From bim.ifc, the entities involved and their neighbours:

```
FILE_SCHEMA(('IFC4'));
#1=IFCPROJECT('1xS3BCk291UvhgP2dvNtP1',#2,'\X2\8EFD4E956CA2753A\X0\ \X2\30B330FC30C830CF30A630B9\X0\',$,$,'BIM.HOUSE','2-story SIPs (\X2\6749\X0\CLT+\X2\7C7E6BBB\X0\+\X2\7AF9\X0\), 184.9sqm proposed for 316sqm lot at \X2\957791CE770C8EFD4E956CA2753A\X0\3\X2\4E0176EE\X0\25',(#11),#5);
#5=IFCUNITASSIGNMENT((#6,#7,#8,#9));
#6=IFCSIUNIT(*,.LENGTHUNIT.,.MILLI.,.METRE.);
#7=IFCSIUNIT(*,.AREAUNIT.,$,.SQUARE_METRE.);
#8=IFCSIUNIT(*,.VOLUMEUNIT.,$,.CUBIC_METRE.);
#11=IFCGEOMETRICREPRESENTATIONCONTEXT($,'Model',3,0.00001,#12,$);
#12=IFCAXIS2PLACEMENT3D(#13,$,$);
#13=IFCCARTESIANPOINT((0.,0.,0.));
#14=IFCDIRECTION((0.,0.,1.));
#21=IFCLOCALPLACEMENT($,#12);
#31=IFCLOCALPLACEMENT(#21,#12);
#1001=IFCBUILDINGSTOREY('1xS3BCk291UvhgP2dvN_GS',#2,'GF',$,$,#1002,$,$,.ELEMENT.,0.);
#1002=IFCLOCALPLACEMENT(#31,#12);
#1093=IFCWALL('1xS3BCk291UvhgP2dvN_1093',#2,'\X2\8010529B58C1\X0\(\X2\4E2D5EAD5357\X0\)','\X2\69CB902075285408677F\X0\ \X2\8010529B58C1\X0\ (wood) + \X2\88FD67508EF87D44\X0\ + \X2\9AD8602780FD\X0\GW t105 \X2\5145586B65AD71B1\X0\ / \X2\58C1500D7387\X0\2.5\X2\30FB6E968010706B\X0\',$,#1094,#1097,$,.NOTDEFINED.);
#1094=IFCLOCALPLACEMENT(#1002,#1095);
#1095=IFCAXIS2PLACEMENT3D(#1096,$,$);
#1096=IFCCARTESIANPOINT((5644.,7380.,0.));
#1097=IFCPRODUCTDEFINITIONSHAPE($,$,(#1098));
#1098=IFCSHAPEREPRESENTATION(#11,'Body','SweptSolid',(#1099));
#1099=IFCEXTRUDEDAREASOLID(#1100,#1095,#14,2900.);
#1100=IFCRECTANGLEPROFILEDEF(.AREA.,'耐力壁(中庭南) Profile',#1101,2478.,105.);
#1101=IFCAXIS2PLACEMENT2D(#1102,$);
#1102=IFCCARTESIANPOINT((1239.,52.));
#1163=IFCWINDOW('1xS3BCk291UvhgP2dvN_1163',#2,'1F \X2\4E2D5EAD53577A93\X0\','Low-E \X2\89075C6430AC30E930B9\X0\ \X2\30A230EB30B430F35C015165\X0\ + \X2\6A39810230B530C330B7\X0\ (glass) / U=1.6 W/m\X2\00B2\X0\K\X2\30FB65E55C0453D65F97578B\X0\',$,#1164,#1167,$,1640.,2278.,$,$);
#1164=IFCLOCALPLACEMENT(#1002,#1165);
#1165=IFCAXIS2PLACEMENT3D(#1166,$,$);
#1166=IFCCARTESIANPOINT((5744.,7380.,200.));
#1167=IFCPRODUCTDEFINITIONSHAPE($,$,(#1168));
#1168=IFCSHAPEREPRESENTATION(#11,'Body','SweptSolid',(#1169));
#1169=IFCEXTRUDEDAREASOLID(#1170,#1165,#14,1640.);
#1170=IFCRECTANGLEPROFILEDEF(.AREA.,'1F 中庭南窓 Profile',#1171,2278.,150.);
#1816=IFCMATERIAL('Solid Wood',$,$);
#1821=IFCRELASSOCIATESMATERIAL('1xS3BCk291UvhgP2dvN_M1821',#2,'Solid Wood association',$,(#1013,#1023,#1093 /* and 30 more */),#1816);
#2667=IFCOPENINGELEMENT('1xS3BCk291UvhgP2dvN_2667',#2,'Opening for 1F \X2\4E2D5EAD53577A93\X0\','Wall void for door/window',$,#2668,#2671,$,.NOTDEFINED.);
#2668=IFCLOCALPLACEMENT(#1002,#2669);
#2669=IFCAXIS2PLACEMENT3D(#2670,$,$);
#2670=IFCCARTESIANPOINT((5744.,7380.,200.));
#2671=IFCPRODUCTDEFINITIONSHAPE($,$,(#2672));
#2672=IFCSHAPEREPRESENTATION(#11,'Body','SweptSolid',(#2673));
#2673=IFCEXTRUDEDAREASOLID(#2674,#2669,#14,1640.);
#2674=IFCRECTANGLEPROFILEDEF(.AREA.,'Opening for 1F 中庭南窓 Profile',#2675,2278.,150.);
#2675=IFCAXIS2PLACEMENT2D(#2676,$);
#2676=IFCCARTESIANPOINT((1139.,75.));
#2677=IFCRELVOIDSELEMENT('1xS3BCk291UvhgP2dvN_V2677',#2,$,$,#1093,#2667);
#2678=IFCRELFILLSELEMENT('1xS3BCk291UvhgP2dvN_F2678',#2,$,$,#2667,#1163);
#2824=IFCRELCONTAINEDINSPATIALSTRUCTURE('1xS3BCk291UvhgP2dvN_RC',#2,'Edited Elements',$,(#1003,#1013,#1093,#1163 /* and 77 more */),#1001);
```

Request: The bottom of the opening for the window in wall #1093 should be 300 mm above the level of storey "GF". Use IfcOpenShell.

```python
import numpy as np
import ifcopenshell
import ifcopenshell.api.geometry
import ifcopenshell.geom
import ifcopenshell.util.element
import ifcopenshell.util.placement
import ifcopenshell.util.shape
import ifcopenshell.util.unit

model = ifcopenshell.open("bim.ifc")
unit_scale = ifcopenshell.util.unit.calculate_unit_scale(model)

window = model.by_guid("1xS3BCk291UvhgP2dvN_1163")
opening = window.FillsVoids[0].RelatingOpeningElement
storey = ifcopenshell.util.element.get_container(window, ifc_class="IfcBuildingStorey")
level = ifcopenshell.util.placement.get_local_placement(storey.ObjectPlacement)[2, 3]

# The opening's origin need not be at the sill, so measure its lowest point.
shape = ifcopenshell.geom.create_shape(ifcopenshell.geom.settings(), opening)
bottom = ifcopenshell.util.shape.get_shape_bottom_elevation(shape, shape.geometry) / unit_scale
dz = level + 0.3 / unit_scale - bottom

shift = np.array([0.0, 0.0, dz])
# The window is not placed relative to its opening, so move both.
for product in (opening, window):
    matrix = ifcopenshell.util.placement.get_local_placement(product.ObjectPlacement)
    matrix[:3, 3] += shift
    ifcopenshell.api.geometry.edit_object_placement(model, product=product, matrix=matrix, is_si=False)

print(f"moved by {dz * unit_scale:+.3f} m")

model.write("bim-out.ifc")
```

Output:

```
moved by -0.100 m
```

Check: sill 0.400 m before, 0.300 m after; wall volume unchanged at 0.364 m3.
